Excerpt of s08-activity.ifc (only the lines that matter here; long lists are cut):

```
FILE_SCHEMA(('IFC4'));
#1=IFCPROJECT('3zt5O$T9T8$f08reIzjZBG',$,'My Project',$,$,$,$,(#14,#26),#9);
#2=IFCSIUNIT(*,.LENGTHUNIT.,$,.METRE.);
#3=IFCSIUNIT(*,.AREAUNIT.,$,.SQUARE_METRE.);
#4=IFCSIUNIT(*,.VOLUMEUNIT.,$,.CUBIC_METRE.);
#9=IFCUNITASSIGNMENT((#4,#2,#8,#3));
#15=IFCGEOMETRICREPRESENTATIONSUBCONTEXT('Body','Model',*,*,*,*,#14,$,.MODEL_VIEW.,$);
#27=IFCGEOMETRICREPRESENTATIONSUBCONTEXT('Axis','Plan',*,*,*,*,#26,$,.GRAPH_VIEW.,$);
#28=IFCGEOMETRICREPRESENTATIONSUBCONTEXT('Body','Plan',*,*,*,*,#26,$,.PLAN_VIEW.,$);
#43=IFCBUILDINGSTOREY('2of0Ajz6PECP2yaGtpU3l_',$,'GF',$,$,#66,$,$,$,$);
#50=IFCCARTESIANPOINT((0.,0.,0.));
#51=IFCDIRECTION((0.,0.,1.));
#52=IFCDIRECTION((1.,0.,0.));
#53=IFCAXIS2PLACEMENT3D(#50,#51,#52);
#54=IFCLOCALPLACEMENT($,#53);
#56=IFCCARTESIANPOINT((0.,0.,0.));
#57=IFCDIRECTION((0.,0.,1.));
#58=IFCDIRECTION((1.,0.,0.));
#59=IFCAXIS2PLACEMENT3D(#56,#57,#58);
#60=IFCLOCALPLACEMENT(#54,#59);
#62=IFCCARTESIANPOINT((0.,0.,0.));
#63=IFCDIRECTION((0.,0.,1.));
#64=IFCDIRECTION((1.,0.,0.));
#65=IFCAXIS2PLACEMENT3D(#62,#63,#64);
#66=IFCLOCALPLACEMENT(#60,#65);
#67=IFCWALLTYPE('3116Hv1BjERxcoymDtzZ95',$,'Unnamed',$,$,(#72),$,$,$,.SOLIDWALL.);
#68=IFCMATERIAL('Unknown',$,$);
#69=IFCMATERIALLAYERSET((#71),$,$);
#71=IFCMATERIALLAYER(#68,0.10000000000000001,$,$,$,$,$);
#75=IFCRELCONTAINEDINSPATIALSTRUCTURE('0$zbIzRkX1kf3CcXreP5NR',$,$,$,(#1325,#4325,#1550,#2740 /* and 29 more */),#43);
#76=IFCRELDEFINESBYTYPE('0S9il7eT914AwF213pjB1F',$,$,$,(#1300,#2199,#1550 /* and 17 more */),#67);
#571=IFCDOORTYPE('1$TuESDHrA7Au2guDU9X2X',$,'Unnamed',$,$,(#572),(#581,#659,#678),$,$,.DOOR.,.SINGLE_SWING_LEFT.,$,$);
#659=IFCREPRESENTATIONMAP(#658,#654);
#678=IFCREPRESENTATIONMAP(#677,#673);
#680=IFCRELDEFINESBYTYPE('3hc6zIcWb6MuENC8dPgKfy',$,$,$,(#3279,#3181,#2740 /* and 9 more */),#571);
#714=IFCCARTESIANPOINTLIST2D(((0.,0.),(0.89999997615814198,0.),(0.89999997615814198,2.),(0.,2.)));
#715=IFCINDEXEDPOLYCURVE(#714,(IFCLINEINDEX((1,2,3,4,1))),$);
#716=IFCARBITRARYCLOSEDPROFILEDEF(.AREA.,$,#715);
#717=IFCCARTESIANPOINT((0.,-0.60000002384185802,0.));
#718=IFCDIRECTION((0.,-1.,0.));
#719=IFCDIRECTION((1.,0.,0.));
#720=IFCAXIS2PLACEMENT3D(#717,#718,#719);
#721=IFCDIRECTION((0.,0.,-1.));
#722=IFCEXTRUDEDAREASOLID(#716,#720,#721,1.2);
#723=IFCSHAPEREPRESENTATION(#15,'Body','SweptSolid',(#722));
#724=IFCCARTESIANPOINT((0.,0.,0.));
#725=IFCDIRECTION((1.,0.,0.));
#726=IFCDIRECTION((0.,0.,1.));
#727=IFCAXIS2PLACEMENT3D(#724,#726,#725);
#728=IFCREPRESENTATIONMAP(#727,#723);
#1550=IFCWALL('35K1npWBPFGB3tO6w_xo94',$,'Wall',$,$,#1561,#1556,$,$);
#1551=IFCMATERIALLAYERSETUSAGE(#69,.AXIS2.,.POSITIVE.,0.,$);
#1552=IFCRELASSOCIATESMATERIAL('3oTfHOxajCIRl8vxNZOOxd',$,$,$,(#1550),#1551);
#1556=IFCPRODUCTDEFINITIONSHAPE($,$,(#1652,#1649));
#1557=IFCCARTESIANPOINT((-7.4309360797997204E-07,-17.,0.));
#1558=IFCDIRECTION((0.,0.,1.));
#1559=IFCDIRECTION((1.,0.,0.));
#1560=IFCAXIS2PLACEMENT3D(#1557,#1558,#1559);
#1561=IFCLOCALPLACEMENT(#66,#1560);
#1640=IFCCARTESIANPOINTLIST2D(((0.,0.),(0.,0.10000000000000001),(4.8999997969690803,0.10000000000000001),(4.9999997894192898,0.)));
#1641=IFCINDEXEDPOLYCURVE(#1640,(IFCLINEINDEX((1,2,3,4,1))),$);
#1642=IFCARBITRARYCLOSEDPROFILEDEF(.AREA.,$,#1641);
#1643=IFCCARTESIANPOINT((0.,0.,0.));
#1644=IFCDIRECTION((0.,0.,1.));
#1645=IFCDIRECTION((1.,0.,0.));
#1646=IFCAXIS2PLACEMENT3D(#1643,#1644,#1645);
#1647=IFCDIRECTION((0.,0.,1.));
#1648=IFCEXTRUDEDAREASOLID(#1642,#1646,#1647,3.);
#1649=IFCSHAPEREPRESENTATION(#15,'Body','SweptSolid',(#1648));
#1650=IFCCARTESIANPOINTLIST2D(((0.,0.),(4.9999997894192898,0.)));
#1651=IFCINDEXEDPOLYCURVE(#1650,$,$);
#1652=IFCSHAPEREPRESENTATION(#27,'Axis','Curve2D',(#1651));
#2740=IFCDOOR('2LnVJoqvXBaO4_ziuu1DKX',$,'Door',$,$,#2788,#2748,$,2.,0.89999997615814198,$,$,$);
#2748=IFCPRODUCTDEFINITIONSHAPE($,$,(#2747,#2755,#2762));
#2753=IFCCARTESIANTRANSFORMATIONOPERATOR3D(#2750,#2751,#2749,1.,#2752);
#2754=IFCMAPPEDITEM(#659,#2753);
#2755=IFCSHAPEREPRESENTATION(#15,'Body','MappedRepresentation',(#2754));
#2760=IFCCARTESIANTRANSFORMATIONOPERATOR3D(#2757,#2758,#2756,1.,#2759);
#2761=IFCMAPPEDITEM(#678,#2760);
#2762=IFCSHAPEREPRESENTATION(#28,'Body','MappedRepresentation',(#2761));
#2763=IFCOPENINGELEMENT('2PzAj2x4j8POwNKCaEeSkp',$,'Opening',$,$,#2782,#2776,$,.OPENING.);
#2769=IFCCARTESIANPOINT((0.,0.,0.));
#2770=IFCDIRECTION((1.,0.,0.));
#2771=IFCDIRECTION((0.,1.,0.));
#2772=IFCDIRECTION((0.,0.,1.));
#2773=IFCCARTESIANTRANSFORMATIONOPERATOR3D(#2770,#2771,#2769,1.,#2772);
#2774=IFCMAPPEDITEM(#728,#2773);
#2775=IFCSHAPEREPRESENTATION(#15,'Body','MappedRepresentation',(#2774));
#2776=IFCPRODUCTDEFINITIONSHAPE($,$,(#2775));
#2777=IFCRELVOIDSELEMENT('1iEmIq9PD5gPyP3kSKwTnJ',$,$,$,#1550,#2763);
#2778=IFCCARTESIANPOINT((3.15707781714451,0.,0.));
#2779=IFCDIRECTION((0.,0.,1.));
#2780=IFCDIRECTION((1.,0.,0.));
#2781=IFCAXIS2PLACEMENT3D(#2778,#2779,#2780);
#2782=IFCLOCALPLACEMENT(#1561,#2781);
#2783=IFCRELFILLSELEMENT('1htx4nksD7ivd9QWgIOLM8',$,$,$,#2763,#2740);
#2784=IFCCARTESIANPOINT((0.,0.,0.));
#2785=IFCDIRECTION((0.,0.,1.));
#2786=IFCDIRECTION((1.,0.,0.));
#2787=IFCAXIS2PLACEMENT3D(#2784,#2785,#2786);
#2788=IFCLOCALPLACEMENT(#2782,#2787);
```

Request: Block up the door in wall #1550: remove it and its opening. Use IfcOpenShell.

```python
import ifcopenshell
import ifcopenshell.api.feature
import ifcopenshell.api.root
import ifcopenshell.geom
import ifcopenshell.util.shape

model = ifcopenshell.open("s08-activity.ifc")
settings = ifcopenshell.geom.settings()


def volume(element):
    """Net volume in cubic metres, openings subtracted."""
    shape = ifcopenshell.geom.create_shape(settings, element)
    return ifcopenshell.util.shape.get_volume(shape.geometry)


door = model.by_guid("2LnVJoqvXBaO4_ziuu1DKX")
opening = door.FillsVoids[0].RelatingOpeningElement
wall = opening.VoidsElements[0].RelatingBuildingElement
before = volume(wall)

ifcopenshell.api.root.remove_product(model, product=door)
ifcopenshell.api.feature.remove_feature(model, feature=opening)

after = volume(wall)

print(f"wall volume {before:.3f} -> {after:.3f} m3")

model.write("s08-activity_edited.ifc")
```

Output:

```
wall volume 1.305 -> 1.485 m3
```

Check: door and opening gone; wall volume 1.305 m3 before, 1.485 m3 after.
